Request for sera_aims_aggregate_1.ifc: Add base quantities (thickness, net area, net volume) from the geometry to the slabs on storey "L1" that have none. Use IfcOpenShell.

First a look at what the model holds.

```python
import ifcopenshell
import ifcopenshell.util.element
import ifcopenshell.util.unit

model = ifcopenshell.open("sera_aims_aggregate_1.ifc")
print(model.schema)
for unit_type in ("LENGTHUNIT", "AREAUNIT", "VOLUMEUNIT"):
    print(unit_type, ifcopenshell.util.unit.calculate_unit_scale(model, unit_type))
storey = next(s for s in model.by_type("IfcBuildingStorey") if s.Name == "L1")
slabs = [e for e in ifcopenshell.util.element.get_decomposition(storey) if e.is_a("IfcSlab")]
for e in sorted(slabs, key=lambda e: e.id()):
    print(e.id(), e.is_a(), e.Name, list(ifcopenshell.util.element.get_psets(e, qtos_only=True)), sep=" | ")
```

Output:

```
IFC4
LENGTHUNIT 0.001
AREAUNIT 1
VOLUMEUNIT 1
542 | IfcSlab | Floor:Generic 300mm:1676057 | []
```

```python
import ifcopenshell
import ifcopenshell.api.pset
import ifcopenshell.geom
import ifcopenshell.util.element
import ifcopenshell.util.shape
import ifcopenshell.util.unit

model = ifcopenshell.open("sera_aims_aggregate_1.ifc")
unit_scale = ifcopenshell.util.unit.calculate_unit_scale(model)
area_scale = ifcopenshell.util.unit.calculate_unit_scale(model, "AREAUNIT")
volume_scale = ifcopenshell.util.unit.calculate_unit_scale(model, "VOLUMEUNIT")
settings = ifcopenshell.geom.settings()

storey = next(s for s in model.by_type("IfcBuildingStorey") if s.Name == "L1")
slabs = [e for e in ifcopenshell.util.element.get_decomposition(storey) if e.is_a("IfcSlab")]

for e in sorted(slabs, key=lambda e: e.id()):
    if ifcopenshell.util.element.get_psets(e, qtos_only=True, should_inherit=False):
        continue
    # Geometry comes back in metres, in the element's own axes.
    shape = ifcopenshell.geom.create_shape(settings, e)
    values = {
        "Width": ifcopenshell.util.shape.get_z(shape.geometry) / unit_scale,
        "NetArea": ifcopenshell.util.shape.get_footprint_area(shape.geometry) / area_scale,
        "NetVolume": ifcopenshell.util.shape.get_volume(shape.geometry) / volume_scale,
    }
    qto = ifcopenshell.api.pset.add_qto(model, product=e, name="Qto_SlabBaseQuantities")
    ifcopenshell.api.pset.edit_qto(model, qto=qto, properties=values)
    print(e.id(), {k: round(v, 3) for k, v in values.items()})

model.write("sera_aims_aggregate_1_v2.ifc")
```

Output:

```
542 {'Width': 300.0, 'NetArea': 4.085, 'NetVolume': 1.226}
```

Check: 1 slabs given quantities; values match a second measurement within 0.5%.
